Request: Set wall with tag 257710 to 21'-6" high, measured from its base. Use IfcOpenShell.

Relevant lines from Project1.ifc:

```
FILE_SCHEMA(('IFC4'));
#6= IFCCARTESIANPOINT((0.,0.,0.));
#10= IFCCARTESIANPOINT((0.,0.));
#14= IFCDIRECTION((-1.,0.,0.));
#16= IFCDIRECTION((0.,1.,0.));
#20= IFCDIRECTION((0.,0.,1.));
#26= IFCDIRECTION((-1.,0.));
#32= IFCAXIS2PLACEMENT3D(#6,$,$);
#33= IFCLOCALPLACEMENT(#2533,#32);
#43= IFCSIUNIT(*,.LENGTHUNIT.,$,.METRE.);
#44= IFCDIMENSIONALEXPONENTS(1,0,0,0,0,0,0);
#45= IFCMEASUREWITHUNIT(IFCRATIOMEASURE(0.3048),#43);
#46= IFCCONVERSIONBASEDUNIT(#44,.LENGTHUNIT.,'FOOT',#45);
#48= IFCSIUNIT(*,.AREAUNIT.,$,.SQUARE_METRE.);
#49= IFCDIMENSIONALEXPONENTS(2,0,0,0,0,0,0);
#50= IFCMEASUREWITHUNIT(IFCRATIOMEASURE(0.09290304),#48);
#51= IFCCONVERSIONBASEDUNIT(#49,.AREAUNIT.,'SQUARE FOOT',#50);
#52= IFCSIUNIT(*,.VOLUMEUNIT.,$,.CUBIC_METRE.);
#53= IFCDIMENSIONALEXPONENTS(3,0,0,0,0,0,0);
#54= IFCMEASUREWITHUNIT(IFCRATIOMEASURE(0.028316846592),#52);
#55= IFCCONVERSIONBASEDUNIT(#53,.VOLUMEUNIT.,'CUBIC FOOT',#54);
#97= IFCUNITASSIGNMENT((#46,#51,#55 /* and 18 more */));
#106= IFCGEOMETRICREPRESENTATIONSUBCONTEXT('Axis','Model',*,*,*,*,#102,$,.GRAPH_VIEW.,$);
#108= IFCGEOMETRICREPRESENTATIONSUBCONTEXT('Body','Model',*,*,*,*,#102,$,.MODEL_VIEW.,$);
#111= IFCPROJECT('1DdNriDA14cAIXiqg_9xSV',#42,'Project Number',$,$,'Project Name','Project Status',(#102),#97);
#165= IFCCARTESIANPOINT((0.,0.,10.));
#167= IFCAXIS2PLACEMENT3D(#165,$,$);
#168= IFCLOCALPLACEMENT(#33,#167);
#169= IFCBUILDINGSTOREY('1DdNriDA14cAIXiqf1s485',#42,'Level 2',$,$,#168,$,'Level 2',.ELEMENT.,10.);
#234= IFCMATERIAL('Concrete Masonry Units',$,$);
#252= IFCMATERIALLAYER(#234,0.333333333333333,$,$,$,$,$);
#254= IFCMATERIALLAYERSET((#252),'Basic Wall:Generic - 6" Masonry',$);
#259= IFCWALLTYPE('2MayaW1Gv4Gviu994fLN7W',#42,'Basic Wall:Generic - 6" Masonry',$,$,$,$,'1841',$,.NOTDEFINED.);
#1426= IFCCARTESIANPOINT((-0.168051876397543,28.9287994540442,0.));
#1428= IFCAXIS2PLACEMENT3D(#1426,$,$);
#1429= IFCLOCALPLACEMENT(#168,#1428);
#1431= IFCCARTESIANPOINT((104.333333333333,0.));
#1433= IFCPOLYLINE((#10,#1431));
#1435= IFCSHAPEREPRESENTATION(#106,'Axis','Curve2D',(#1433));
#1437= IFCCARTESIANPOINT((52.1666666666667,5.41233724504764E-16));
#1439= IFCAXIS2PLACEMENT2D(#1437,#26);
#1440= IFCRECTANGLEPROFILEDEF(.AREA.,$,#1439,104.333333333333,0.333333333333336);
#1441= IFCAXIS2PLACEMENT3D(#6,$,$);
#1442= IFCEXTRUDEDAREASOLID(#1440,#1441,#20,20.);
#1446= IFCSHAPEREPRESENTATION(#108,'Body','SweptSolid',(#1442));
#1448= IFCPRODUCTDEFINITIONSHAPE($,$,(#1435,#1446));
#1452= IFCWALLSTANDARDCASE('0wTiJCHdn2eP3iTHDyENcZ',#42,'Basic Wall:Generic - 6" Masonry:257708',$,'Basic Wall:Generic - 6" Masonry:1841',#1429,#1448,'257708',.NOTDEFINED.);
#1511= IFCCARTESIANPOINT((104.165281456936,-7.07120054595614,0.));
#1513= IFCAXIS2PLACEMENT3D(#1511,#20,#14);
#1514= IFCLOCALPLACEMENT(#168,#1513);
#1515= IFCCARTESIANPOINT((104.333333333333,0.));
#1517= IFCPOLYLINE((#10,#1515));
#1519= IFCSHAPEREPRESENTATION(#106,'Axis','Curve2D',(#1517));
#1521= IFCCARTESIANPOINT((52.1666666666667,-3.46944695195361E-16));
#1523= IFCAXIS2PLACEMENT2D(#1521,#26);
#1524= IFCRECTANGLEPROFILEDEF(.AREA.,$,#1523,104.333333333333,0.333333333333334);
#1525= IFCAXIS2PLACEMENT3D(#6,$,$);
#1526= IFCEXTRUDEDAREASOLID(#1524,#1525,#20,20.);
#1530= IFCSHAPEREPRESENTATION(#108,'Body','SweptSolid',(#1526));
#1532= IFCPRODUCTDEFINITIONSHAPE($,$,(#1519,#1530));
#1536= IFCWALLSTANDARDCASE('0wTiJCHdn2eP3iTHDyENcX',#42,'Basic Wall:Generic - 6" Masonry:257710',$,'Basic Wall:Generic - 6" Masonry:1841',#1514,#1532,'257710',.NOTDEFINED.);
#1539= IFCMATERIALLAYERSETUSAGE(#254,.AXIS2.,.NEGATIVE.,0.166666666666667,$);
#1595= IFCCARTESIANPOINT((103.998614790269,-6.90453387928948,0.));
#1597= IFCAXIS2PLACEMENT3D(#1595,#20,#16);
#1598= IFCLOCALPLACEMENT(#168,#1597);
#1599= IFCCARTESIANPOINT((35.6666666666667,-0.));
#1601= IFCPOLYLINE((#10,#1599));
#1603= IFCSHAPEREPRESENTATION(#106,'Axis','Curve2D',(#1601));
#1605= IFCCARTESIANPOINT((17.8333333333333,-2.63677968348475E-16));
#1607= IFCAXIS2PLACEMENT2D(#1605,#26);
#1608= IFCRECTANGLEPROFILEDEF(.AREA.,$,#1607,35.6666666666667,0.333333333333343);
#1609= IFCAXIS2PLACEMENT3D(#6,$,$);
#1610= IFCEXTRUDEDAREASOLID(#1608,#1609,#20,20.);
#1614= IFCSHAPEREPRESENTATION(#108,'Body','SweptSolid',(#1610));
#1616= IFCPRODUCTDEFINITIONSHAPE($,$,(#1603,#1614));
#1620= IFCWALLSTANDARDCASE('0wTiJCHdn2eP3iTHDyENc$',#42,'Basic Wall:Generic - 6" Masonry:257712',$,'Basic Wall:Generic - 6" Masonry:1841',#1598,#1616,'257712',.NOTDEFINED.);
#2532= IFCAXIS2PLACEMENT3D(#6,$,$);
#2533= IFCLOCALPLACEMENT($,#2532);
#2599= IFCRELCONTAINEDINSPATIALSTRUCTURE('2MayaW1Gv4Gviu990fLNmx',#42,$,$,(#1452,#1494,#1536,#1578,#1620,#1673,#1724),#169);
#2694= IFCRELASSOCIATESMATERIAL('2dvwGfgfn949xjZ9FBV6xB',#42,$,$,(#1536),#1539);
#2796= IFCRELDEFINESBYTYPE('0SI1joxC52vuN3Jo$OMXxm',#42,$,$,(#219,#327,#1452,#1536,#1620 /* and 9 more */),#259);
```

```python
import ifcopenshell
import ifcopenshell.geom
import ifcopenshell.util.representation
import ifcopenshell.util.shape
import ifcopenshell.util.unit

model = ifcopenshell.open("Project1.ifc")
unit_scale = ifcopenshell.util.unit.calculate_unit_scale(model)
settings = ifcopenshell.geom.settings()


def volume(element):
    """Net volume in cubic metres, openings subtracted."""
    shape = ifcopenshell.geom.create_shape(settings, element)
    return ifcopenshell.util.shape.get_volume(shape.geometry)


wall = model.by_guid("0wTiJCHdn2eP3iTHDyENcX")
before = volume(wall)

body = ifcopenshell.util.representation.get_representation(wall, "Model", "Body")
solid = body.Items[0]
old_height = solid.Depth
solid.Depth = 258 * 0.0254 / unit_scale
after = volume(wall)

print(f"height {old_height:g} -> {solid.Depth:g}, volume {before:.3f} -> {after:.3f} m3")

model.write("Project1_updated.ifc")
```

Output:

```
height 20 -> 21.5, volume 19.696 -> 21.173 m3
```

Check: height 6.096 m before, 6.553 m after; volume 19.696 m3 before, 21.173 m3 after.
